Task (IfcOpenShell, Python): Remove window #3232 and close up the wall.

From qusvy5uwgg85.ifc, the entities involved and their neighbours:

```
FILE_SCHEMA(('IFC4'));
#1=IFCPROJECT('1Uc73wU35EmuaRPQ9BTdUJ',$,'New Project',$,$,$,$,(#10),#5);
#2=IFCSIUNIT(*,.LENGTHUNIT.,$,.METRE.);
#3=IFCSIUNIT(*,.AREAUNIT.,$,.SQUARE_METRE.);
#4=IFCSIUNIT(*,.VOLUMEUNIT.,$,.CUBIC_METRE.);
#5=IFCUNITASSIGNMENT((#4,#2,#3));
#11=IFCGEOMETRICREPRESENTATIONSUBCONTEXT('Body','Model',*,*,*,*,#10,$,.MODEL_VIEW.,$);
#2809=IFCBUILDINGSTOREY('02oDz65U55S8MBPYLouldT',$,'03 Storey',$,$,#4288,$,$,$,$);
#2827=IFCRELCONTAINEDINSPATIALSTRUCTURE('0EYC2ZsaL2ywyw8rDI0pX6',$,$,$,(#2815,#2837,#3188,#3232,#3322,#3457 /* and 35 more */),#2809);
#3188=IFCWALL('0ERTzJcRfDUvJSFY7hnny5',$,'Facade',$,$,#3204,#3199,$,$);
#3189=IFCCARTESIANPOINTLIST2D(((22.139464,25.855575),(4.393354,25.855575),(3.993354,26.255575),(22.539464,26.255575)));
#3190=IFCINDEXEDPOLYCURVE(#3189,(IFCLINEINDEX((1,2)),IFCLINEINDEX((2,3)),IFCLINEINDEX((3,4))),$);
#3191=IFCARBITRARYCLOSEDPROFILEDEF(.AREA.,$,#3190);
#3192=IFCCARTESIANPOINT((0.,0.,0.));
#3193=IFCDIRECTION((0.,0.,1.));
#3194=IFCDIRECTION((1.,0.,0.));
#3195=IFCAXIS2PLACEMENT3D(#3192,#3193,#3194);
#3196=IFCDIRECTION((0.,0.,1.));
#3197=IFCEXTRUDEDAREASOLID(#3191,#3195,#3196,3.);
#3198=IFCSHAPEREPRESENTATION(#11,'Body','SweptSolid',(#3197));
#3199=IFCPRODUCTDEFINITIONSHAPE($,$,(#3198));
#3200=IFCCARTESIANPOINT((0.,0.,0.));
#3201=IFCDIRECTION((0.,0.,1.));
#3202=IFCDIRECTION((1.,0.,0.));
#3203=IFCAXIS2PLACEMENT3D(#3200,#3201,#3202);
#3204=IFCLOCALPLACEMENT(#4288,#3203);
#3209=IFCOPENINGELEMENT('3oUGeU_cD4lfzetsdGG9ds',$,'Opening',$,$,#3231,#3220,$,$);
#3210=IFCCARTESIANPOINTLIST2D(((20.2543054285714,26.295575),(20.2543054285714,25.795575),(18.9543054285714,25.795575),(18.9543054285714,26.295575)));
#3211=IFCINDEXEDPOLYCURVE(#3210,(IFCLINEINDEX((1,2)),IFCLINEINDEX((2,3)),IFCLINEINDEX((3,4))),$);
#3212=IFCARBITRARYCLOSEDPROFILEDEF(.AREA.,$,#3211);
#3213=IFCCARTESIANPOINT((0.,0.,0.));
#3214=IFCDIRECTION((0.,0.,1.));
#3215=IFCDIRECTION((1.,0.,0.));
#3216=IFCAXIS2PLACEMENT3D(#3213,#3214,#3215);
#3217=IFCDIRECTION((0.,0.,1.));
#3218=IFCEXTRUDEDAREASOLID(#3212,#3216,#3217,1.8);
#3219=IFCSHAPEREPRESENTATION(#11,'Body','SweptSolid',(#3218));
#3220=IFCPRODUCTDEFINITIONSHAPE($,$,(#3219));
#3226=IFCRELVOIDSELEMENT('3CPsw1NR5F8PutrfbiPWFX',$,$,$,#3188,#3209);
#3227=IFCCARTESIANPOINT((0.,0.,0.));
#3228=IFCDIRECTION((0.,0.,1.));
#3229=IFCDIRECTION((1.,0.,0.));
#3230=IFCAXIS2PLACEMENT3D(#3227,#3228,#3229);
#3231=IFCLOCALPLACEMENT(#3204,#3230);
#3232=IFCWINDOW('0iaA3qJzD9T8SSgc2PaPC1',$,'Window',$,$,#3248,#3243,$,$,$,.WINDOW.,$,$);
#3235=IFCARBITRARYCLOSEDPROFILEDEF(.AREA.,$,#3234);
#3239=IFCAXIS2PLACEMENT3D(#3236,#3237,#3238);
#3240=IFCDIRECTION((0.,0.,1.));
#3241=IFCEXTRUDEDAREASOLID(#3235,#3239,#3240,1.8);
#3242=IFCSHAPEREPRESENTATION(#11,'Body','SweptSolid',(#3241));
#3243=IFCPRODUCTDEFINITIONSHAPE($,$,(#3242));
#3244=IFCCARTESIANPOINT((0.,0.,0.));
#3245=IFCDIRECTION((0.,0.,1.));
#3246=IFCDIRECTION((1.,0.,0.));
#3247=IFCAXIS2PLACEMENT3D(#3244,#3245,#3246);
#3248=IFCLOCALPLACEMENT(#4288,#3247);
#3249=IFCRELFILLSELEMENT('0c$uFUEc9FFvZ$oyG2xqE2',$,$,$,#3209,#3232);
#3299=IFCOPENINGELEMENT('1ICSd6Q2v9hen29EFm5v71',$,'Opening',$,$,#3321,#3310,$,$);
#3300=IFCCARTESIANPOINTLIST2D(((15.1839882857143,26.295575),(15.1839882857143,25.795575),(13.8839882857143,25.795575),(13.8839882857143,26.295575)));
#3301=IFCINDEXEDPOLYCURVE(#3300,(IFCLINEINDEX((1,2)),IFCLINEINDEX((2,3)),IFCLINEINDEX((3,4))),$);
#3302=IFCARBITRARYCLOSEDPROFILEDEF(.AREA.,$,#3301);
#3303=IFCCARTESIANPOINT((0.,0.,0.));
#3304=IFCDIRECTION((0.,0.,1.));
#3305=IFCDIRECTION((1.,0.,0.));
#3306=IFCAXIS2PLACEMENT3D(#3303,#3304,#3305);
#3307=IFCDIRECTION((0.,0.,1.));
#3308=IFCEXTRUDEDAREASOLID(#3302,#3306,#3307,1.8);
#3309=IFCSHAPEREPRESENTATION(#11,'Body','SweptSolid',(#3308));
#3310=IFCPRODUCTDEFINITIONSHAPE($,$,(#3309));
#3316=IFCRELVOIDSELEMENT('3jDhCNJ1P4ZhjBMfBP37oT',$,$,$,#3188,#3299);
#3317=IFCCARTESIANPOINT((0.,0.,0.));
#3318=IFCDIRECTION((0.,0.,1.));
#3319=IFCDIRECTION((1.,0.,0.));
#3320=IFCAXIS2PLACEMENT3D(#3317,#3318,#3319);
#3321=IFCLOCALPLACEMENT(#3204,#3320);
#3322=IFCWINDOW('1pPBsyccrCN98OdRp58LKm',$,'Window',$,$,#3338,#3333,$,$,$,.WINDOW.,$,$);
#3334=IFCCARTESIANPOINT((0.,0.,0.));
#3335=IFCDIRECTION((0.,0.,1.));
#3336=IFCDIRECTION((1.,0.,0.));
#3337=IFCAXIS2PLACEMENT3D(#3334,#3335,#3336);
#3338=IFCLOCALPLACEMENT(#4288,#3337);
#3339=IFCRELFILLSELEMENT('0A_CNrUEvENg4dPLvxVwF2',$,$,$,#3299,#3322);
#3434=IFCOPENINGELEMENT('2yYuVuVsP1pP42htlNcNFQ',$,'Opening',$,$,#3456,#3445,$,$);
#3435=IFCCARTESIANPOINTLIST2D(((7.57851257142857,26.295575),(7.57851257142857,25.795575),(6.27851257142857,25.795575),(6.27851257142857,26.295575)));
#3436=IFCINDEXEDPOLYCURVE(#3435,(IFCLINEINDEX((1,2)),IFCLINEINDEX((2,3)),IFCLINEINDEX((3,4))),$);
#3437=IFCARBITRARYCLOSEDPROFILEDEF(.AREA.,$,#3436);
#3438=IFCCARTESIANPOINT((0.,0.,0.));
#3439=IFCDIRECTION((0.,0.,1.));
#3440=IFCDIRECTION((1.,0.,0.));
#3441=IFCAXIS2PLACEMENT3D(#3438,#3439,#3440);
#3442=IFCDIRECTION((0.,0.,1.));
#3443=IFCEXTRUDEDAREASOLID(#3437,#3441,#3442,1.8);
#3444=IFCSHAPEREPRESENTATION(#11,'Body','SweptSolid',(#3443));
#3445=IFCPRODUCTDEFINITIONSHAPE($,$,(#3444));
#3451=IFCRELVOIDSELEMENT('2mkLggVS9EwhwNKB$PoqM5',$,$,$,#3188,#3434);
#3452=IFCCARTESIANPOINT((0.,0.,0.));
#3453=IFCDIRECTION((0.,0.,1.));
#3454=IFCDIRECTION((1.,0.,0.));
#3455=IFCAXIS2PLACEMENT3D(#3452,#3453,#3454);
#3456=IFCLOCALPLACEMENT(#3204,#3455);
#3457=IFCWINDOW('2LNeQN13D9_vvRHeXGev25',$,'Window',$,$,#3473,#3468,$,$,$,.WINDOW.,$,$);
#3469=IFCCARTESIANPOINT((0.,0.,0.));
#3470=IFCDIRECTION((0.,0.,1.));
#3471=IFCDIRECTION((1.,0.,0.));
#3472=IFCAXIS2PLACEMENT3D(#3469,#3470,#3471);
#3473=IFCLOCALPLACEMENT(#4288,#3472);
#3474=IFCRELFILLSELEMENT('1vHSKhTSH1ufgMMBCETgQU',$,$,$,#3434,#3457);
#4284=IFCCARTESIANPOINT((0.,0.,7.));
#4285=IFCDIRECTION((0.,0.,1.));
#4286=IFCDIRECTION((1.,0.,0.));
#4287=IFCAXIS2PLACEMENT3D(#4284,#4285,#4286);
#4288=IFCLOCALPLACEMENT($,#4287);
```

```python
import ifcopenshell
import ifcopenshell.api.feature
import ifcopenshell.api.root
import ifcopenshell.geom
import ifcopenshell.util.shape

model = ifcopenshell.open("qusvy5uwgg85.ifc")
settings = ifcopenshell.geom.settings()


def volume(element):
    """Net volume in cubic metres, openings subtracted."""
    shape = ifcopenshell.geom.create_shape(settings, element)
    return ifcopenshell.util.shape.get_volume(shape.geometry)


window = model.by_id(3232)
opening = window.FillsVoids[0].RelatingOpeningElement
wall = opening.VoidsElements[0].RelatingBuildingElement
before = volume(wall)

ifcopenshell.api.root.remove_product(model, product=window)
ifcopenshell.api.feature.remove_feature(model, feature=opening)

after = volume(wall)

print(f"wall volume {before:.3f} -> {after:.3f} m3")

model.write("qusvy5uwgg85_updated.ifc")
```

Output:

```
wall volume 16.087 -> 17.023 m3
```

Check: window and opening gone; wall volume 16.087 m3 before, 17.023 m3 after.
